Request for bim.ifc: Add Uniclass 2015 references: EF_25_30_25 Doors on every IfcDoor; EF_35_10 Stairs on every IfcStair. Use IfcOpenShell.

First a look at what the model holds.

```python
import ifcopenshell

model = ifcopenshell.open("bim.ifc")
print(model.schema)
print("classifications:", [c.Name for c in model.by_type("IfcClassification")])
for ifc_class in ("IfcDoor", "IfcRoof", "IfcStair", "IfcWall", "IfcWindow"):
    print(ifc_class, len(model.by_type(ifc_class)))
```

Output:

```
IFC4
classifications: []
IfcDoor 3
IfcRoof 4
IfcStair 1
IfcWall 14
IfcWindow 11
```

```python
import ifcopenshell
import ifcopenshell.api.classification

model = ifcopenshell.open("bim.ifc")

system = ifcopenshell.api.classification.add_classification(model, classification="Uniclass 2015")

codes = {
    "IfcDoor": ("EF_25_30_25", "Doors"),
    "IfcStair": ("EF_35_10", "Stairs"),
}
for ifc_class, (code, name) in codes.items():
    products = model.by_type(ifc_class)
    ifcopenshell.api.classification.add_reference(
        model, products=products, classification=system, identification=code, name=name
    )
    print(code, len(products))

model.write("bim_rev.ifc")
```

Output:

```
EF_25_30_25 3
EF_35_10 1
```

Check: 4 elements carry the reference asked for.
